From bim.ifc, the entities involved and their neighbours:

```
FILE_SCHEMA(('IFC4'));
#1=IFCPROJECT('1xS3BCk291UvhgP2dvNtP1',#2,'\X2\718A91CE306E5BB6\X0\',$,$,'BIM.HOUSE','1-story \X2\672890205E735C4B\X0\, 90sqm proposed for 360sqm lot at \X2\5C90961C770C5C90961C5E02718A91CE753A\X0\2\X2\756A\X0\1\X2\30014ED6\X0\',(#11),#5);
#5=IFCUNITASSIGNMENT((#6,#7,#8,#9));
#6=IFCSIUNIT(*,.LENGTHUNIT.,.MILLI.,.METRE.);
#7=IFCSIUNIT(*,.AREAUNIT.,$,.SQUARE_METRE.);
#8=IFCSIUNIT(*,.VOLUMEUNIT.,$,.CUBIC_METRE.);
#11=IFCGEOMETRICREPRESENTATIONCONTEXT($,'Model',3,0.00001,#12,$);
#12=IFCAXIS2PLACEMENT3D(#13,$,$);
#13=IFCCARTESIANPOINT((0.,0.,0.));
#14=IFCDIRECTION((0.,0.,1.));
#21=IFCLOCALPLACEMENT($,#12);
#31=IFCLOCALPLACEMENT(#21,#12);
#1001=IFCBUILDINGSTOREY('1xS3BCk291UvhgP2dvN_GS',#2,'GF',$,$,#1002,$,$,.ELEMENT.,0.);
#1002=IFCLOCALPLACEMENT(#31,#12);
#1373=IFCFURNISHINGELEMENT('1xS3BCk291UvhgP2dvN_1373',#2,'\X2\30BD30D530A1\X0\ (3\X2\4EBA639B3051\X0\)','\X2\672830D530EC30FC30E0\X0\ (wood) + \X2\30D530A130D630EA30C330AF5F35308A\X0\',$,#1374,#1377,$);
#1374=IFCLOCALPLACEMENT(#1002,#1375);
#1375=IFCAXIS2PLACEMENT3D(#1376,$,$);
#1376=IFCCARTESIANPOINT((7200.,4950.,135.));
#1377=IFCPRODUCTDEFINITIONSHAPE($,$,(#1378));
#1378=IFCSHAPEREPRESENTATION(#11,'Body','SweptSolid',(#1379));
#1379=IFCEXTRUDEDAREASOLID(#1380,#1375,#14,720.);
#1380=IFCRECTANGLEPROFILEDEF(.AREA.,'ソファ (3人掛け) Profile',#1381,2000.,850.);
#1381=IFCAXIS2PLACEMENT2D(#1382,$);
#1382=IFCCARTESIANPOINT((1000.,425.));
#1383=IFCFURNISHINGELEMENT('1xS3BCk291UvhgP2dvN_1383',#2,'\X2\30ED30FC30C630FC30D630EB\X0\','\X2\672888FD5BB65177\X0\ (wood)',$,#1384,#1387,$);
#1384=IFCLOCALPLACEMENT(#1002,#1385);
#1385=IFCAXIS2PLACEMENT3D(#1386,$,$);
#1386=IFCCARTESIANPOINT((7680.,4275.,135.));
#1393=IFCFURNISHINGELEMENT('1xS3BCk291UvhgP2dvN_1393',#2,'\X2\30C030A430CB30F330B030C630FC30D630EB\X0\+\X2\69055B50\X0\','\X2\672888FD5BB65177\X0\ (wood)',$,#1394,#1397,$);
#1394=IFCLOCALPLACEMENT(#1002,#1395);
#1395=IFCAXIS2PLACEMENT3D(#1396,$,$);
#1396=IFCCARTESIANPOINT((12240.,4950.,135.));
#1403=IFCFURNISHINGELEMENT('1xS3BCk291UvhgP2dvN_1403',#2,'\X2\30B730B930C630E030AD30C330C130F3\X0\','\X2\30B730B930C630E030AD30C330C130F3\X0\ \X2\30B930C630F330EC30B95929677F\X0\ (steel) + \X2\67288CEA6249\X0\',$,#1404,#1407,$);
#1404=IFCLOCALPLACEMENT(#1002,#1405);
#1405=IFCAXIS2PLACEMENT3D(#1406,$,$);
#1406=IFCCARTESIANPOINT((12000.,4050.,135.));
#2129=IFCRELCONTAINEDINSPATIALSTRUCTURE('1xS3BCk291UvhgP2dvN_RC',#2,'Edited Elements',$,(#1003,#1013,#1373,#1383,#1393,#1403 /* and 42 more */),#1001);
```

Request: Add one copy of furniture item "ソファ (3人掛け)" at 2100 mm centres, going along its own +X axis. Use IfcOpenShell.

```python
import ifcopenshell
import ifcopenshell.api.geometry
import ifcopenshell.api.root
import ifcopenshell.util.element
import ifcopenshell.util.placement
import ifcopenshell.util.unit

model = ifcopenshell.open("bim.ifc")
unit_scale = ifcopenshell.util.unit.calculate_unit_scale(model)


def reuse_history(source, copy):
    """copy_class also copies each property set's owner history, people and application; keep the originals."""
    for rel in copy.IsDefinedBy:
        if rel.is_a("IfcRelDefinesByProperties") and (history := rel.RelatingPropertyDefinition.OwnerHistory):
            rel.RelatingPropertyDefinition.OwnerHistory = source.OwnerHistory
            ifcopenshell.util.element.remove_deep2(model, history)


source = model.by_id(1373)
base = ifcopenshell.util.placement.get_local_placement(source.ObjectPlacement)
step = base[:3, 0] * 2.1 / unit_scale

for i in range(1, 2):
    copy = ifcopenshell.api.root.copy_class(model, product=source)
    copy.Representation = ifcopenshell.util.element.copy_deep(
        model, source.Representation, exclude=["IfcGeometricRepresentationContext", "IfcRepresentationMap"]
    )
    reuse_history(source, copy)
    matrix = base.copy()
    matrix[:3, 3] += i * step
    print("added at", matrix[:3, 3].round(3) + 0.0)
    ifcopenshell.api.geometry.edit_object_placement(model, product=copy, matrix=matrix, is_si=False)

model.write("bim_updated.ifc")
```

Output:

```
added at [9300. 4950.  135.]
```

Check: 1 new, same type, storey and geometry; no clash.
